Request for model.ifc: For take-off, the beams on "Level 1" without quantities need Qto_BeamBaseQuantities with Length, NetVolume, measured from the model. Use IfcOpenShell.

First a look at what the model holds.

```python
import ifcopenshell
import ifcopenshell.util.element
import ifcopenshell.util.unit

model = ifcopenshell.open("model.ifc")
print(model.schema)
for unit_type in ("LENGTHUNIT", "AREAUNIT", "VOLUMEUNIT"):
    print(unit_type, ifcopenshell.util.unit.calculate_unit_scale(model, unit_type))
storey = next(s for s in model.by_type("IfcBuildingStorey") if s.Name == "Level 1")
beams = [e for e in ifcopenshell.util.element.get_decomposition(storey) if e.is_a("IfcBeam")]
for e in sorted(beams, key=lambda e: e.id()):
    print(e.id(), e.is_a(), e.Name, list(ifcopenshell.util.element.get_psets(e, qtos_only=True)), sep=" | ")
```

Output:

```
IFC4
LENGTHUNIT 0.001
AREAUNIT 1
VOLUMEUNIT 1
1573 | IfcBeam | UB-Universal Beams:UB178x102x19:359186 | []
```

```python
import ifcopenshell
import ifcopenshell.api.pset
import ifcopenshell.geom
import ifcopenshell.util.element
import ifcopenshell.util.shape
import ifcopenshell.util.unit

model = ifcopenshell.open("model.ifc")
unit_scale = ifcopenshell.util.unit.calculate_unit_scale(model)
volume_scale = ifcopenshell.util.unit.calculate_unit_scale(model, "VOLUMEUNIT")
settings = ifcopenshell.geom.settings()

storey = next(s for s in model.by_type("IfcBuildingStorey") if s.Name == "Level 1")
beams = [e for e in ifcopenshell.util.element.get_decomposition(storey) if e.is_a("IfcBeam")]

for e in sorted(beams, key=lambda e: e.id()):
    if ifcopenshell.util.element.get_psets(e, qtos_only=True, should_inherit=False):
        continue
    # Geometry comes back in metres, in the element's own axes.
    shape = ifcopenshell.geom.create_shape(settings, e)
    values = {
        "Length": ifcopenshell.util.shape.get_max_xyz(shape.geometry) / unit_scale,
        "NetVolume": ifcopenshell.util.shape.get_volume(shape.geometry) / volume_scale,
    }
    qto = ifcopenshell.api.pset.add_qto(model, product=e, name="Qto_BeamBaseQuantities")
    ifcopenshell.api.pset.edit_qto(model, qto=qto, properties=values)
    print(e.id(), {k: round(v, 3) for k, v in values.items()})

model.write("model_edited.ifc")
```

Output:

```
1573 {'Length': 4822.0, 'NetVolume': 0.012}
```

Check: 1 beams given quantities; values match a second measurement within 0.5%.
